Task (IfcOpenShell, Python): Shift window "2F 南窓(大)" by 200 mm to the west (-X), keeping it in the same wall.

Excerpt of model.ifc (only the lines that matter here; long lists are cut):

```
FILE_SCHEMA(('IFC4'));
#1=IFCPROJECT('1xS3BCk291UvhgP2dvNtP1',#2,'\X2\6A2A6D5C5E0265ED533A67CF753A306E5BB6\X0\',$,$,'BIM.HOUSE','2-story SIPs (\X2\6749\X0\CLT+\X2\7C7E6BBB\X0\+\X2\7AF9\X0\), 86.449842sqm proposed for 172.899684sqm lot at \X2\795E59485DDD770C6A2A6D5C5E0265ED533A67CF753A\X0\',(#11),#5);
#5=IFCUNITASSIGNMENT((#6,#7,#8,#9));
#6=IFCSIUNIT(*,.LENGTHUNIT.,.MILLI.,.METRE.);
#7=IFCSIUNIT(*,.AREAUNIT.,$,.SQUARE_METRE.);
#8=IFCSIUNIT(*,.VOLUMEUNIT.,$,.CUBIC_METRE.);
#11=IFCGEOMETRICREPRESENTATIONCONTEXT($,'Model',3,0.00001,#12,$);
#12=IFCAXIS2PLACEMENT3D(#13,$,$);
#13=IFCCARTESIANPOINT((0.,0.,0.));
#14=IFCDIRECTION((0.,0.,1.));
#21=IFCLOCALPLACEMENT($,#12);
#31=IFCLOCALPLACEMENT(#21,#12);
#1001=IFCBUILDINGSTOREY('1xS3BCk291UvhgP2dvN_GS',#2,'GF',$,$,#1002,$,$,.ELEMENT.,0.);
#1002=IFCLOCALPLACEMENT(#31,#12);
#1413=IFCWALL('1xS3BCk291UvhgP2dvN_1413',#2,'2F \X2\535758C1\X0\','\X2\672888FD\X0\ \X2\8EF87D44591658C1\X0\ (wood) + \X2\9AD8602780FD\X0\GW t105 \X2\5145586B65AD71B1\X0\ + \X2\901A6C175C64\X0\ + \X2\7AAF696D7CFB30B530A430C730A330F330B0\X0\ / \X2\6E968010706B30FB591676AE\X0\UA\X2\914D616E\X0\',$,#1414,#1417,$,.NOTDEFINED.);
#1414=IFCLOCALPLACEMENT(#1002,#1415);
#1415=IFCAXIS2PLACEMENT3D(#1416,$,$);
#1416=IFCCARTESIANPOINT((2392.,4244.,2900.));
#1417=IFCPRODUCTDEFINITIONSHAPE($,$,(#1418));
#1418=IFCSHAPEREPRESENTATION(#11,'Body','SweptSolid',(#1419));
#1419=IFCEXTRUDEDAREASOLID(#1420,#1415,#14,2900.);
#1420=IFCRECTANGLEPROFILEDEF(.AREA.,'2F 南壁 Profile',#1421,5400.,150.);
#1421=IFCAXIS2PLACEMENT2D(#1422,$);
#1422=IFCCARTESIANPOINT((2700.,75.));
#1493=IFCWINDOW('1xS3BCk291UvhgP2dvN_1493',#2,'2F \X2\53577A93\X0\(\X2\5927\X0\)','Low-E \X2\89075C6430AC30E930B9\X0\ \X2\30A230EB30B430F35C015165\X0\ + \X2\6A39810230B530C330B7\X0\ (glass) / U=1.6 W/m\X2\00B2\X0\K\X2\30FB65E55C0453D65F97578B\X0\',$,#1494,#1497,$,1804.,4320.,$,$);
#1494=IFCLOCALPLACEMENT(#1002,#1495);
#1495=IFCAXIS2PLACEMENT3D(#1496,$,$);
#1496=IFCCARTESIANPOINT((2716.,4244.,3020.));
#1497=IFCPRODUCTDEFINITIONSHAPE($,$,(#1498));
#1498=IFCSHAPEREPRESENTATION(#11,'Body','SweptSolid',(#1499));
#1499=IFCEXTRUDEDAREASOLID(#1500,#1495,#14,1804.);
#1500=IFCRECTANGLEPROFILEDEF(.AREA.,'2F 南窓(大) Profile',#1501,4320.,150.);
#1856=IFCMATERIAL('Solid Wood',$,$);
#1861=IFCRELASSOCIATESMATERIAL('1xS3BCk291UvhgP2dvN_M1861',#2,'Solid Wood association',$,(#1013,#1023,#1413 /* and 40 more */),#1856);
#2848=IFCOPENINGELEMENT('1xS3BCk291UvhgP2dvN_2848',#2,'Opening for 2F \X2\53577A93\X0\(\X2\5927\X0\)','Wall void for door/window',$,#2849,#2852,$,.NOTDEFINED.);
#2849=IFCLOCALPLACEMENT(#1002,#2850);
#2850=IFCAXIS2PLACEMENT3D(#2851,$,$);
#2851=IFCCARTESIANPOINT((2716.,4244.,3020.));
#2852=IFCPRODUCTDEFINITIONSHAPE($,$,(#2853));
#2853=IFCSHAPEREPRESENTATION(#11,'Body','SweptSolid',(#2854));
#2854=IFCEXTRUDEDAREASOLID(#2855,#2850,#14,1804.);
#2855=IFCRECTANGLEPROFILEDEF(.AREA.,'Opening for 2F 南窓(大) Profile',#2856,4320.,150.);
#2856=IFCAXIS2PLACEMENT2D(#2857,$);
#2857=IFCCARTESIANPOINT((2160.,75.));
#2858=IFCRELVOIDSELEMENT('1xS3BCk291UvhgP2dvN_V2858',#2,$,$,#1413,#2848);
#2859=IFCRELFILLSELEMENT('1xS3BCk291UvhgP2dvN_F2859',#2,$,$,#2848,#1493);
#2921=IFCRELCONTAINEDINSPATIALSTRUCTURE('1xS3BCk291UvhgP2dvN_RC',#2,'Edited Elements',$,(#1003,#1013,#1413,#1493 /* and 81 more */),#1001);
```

```python
import ifcopenshell
import ifcopenshell.api.geometry
import ifcopenshell.util.placement
import ifcopenshell.util.unit

model = ifcopenshell.open("model.ifc")
unit_scale = ifcopenshell.util.unit.calculate_unit_scale(model)

window = model.by_id(1493)
opening = window.FillsVoids[0].RelatingOpeningElement
wall = opening.VoidsElements[0].RelatingBuildingElement

wall_matrix = ifcopenshell.util.placement.get_local_placement(wall.ObjectPlacement)
shift = wall_matrix[:3, 0] * -0.2 / unit_scale
before = ifcopenshell.util.placement.get_local_placement(window.ObjectPlacement)[:3, 3].copy()

# The window is not placed relative to its opening, so move both.
for product in (opening, window):
    matrix = ifcopenshell.util.placement.get_local_placement(product.ObjectPlacement)
    matrix[:3, 3] += shift
    ifcopenshell.api.geometry.edit_object_placement(model, product=product, matrix=matrix, is_si=False)

after = ifcopenshell.util.placement.get_local_placement(window.ObjectPlacement)[:3, 3]
print("window moved by", (after - before).round(3) + 0.0)

model.write("model-out.ifc")
```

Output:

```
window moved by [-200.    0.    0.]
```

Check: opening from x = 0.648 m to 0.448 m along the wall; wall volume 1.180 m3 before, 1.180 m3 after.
